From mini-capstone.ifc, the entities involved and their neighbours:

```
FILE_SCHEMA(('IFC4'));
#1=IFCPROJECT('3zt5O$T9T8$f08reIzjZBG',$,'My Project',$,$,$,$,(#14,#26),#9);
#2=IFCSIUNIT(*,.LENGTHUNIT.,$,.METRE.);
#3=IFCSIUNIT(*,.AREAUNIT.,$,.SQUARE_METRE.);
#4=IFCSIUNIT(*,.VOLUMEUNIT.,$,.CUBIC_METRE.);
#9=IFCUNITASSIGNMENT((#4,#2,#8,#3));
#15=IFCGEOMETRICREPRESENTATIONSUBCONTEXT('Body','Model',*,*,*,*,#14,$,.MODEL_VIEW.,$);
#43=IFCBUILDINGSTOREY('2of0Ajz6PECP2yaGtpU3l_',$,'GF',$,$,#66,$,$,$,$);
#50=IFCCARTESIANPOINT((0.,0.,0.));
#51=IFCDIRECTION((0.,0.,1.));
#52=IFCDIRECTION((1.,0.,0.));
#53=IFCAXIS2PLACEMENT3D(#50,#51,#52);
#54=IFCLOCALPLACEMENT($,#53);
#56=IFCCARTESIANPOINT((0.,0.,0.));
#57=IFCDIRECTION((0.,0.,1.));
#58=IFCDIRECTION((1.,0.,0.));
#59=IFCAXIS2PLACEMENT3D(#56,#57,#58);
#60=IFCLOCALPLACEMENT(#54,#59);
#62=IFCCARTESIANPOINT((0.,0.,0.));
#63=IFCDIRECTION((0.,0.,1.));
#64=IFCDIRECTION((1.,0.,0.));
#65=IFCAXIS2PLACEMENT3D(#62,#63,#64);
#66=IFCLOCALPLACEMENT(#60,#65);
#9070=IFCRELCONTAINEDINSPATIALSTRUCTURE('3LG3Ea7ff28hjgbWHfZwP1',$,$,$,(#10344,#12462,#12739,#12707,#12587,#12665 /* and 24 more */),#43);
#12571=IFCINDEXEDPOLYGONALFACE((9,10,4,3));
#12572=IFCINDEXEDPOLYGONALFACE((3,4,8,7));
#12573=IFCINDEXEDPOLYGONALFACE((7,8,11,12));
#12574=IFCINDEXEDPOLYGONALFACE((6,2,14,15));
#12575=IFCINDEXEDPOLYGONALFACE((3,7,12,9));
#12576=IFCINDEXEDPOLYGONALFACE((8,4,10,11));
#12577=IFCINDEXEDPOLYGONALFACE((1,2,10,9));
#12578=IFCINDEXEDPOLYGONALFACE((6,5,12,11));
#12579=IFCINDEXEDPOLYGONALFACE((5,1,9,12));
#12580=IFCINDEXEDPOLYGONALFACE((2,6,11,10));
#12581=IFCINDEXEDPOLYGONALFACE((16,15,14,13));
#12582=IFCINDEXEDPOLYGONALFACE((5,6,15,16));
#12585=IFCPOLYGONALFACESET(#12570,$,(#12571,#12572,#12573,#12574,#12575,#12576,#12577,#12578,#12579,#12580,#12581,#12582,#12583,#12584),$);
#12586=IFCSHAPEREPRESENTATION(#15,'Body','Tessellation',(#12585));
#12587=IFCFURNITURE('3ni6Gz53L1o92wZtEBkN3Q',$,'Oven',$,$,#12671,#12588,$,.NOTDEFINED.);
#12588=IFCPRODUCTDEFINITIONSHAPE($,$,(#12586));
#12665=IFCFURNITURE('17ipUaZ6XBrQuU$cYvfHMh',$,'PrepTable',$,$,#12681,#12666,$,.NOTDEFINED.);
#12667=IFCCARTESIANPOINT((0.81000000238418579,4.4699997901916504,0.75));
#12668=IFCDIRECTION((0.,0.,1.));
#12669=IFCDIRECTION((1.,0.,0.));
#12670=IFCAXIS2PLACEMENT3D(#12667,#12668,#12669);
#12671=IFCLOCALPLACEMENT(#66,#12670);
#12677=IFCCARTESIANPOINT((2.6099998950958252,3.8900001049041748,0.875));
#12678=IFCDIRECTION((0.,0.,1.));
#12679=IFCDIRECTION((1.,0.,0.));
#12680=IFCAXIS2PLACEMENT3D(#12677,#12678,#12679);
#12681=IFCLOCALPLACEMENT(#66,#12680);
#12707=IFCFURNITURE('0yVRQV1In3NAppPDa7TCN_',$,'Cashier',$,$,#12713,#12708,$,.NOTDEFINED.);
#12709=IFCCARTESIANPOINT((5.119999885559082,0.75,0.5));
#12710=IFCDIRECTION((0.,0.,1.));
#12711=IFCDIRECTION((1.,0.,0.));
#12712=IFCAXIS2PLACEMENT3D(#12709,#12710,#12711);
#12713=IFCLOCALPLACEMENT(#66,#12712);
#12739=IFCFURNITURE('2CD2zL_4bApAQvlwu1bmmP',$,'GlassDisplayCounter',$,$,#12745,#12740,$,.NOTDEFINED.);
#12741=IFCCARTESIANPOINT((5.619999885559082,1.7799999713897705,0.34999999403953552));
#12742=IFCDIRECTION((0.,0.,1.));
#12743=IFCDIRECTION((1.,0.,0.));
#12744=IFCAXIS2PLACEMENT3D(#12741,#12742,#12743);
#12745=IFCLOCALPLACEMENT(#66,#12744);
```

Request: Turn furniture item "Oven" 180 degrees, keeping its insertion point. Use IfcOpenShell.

```python
import ifcopenshell
import ifcopenshell.api.geometry
import ifcopenshell.util.placement

model = ifcopenshell.open("mini-capstone.ifc")

item = model.by_id(12587)
matrix = ifcopenshell.util.placement.get_local_placement(item.ObjectPlacement)
matrix = matrix @ ifcopenshell.util.placement.rotation(180, "Z")
ifcopenshell.api.geometry.edit_object_placement(model, product=item, matrix=matrix, is_si=False)

print(ifcopenshell.util.placement.get_local_placement(item.ObjectPlacement).round(3) + 0.0)

model.write("mini-capstone_rev.ifc")
```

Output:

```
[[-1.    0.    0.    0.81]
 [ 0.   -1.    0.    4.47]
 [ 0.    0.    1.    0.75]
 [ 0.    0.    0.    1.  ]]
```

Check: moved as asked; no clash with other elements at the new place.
